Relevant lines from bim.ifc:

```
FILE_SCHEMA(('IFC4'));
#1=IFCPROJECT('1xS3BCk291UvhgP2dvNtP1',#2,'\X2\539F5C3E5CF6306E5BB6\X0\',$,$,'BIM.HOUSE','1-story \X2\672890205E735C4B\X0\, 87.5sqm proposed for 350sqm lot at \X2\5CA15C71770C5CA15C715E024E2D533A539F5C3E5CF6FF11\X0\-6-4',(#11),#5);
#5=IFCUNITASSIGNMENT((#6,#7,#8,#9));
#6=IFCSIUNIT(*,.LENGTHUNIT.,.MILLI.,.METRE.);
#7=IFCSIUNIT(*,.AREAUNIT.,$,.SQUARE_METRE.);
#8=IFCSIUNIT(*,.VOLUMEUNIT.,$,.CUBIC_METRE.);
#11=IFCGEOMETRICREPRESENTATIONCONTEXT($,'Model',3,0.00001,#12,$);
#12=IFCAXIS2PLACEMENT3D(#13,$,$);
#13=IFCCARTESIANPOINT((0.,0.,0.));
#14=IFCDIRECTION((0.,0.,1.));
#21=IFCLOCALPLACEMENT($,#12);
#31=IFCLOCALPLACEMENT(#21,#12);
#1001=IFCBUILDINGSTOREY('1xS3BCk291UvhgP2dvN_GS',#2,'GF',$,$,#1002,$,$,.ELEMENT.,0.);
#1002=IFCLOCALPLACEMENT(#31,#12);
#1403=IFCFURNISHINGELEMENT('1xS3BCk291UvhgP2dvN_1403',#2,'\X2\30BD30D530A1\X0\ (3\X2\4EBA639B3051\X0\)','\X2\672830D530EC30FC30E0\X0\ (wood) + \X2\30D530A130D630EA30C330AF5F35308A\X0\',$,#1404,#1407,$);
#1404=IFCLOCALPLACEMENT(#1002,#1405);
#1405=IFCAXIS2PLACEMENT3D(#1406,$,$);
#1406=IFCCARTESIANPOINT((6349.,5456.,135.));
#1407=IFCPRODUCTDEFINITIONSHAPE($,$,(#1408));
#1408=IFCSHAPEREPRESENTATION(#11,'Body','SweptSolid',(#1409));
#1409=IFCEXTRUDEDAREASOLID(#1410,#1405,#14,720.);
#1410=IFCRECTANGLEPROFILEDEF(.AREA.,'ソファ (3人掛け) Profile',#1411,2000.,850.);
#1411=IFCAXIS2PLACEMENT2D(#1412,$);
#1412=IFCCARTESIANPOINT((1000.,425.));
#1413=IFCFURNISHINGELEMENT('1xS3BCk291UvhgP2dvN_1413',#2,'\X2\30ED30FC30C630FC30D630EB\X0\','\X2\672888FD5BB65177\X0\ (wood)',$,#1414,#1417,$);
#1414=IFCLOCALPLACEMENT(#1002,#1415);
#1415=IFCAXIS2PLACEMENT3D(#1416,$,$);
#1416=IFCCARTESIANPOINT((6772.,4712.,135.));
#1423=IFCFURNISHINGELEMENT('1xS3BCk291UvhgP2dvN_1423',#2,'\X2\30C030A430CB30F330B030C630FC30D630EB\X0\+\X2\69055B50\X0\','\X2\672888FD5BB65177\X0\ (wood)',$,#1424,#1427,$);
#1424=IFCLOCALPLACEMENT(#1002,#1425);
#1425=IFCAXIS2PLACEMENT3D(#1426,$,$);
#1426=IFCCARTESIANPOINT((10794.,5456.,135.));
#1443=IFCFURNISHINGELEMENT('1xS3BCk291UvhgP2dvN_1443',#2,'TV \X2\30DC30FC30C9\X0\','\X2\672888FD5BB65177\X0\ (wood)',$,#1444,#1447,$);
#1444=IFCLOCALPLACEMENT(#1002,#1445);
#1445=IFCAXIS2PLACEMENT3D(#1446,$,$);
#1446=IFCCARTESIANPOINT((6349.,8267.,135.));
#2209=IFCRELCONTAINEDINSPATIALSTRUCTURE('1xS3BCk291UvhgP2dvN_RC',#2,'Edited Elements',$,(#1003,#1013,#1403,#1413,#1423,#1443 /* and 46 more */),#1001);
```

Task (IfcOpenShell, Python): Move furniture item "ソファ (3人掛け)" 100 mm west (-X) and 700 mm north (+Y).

```python
import ifcopenshell
import ifcopenshell.api.geometry
import ifcopenshell.util.placement

model = ifcopenshell.open("bim.ifc")

item = model.by_guid("1xS3BCk291UvhgP2dvN_1403")
matrix = ifcopenshell.util.placement.get_local_placement(item.ObjectPlacement)
matrix[0, 3] -= 100.0
matrix[1, 3] += 700.0
ifcopenshell.api.geometry.edit_object_placement(model, product=item, matrix=matrix, is_si=False)

print(ifcopenshell.util.placement.get_local_placement(item.ObjectPlacement).round(3) + 0.0)

model.write("bim-out.ifc")
```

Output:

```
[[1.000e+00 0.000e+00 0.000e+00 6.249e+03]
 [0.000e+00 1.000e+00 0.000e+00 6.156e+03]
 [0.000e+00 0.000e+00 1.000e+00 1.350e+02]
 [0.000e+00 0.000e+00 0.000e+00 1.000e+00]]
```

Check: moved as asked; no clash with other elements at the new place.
